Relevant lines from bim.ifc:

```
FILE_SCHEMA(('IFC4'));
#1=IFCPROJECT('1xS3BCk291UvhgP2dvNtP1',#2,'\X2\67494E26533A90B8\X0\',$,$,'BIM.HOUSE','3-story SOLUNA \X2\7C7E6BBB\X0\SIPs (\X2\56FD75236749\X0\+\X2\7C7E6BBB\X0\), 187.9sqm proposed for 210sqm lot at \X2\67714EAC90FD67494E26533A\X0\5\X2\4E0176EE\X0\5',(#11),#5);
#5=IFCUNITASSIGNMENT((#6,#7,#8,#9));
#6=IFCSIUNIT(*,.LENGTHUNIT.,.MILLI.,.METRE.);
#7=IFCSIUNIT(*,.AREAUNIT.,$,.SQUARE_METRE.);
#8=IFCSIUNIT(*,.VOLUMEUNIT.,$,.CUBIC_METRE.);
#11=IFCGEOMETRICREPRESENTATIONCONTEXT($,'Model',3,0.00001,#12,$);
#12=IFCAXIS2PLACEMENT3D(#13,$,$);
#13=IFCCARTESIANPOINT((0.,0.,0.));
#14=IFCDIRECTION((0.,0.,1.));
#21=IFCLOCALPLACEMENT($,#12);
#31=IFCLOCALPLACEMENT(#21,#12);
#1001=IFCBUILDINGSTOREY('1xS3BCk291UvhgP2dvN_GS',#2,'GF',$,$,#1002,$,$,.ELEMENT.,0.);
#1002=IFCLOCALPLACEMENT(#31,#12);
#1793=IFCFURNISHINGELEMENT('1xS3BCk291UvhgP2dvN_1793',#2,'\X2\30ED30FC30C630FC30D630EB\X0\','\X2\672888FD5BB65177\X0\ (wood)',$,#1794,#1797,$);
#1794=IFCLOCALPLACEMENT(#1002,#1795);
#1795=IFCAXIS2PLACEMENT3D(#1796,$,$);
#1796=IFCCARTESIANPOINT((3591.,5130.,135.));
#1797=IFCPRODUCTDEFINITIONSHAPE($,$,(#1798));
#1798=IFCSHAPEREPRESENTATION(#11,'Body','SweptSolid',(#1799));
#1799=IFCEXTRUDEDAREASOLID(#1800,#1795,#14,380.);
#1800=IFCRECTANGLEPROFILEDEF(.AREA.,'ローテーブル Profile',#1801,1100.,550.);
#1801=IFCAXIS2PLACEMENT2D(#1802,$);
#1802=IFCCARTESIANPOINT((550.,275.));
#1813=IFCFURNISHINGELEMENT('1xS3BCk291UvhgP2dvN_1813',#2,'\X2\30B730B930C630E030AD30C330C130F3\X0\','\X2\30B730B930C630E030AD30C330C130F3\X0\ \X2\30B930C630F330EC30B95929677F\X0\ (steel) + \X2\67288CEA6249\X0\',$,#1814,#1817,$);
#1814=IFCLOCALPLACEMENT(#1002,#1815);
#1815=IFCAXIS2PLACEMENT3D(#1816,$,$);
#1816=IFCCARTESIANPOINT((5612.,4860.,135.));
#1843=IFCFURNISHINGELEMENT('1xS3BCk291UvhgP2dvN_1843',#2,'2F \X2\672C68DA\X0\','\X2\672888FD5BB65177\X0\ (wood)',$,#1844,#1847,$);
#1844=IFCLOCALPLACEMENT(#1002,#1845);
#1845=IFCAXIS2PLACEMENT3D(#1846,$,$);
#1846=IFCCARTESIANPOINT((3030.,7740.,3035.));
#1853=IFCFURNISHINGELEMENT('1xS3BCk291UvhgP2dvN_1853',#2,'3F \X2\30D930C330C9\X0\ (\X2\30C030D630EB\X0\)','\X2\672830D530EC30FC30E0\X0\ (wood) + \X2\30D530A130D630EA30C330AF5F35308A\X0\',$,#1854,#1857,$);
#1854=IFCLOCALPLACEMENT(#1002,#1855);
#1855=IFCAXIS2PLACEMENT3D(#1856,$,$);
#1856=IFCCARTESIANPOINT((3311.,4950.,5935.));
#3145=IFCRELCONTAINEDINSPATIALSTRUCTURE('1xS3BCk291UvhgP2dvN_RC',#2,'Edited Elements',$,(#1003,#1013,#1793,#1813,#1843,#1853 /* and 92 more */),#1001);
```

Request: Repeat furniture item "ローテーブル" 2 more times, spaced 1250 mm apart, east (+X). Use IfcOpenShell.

```python
import numpy as np
import ifcopenshell
import ifcopenshell.api.geometry
import ifcopenshell.api.root
import ifcopenshell.util.element
import ifcopenshell.util.placement
import ifcopenshell.util.unit

model = ifcopenshell.open("bim.ifc")
unit_scale = ifcopenshell.util.unit.calculate_unit_scale(model)


def reuse_history(source, copy):
    """copy_class also copies each property set's owner history, people and application; keep the originals."""
    for rel in copy.IsDefinedBy:
        if rel.is_a("IfcRelDefinesByProperties") and (history := rel.RelatingPropertyDefinition.OwnerHistory):
            rel.RelatingPropertyDefinition.OwnerHistory = source.OwnerHistory
            ifcopenshell.util.element.remove_deep2(model, history)


source = model.by_id(1793)
base = ifcopenshell.util.placement.get_local_placement(source.ObjectPlacement)
step = np.array([1.0, 0.0, 0.0]) * 1.25 / unit_scale

for i in range(1, 3):
    copy = ifcopenshell.api.root.copy_class(model, product=source)
    copy.Representation = ifcopenshell.util.element.copy_deep(
        model, source.Representation, exclude=["IfcGeometricRepresentationContext", "IfcRepresentationMap"]
    )
    reuse_history(source, copy)
    matrix = base.copy()
    matrix[:3, 3] += i * step
    print("added at", matrix[:3, 3].round(3) + 0.0)
    ifcopenshell.api.geometry.edit_object_placement(model, product=copy, matrix=matrix, is_si=False)

model.write("bim_rev.ifc")
```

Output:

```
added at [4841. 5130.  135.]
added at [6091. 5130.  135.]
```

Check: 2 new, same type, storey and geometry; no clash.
